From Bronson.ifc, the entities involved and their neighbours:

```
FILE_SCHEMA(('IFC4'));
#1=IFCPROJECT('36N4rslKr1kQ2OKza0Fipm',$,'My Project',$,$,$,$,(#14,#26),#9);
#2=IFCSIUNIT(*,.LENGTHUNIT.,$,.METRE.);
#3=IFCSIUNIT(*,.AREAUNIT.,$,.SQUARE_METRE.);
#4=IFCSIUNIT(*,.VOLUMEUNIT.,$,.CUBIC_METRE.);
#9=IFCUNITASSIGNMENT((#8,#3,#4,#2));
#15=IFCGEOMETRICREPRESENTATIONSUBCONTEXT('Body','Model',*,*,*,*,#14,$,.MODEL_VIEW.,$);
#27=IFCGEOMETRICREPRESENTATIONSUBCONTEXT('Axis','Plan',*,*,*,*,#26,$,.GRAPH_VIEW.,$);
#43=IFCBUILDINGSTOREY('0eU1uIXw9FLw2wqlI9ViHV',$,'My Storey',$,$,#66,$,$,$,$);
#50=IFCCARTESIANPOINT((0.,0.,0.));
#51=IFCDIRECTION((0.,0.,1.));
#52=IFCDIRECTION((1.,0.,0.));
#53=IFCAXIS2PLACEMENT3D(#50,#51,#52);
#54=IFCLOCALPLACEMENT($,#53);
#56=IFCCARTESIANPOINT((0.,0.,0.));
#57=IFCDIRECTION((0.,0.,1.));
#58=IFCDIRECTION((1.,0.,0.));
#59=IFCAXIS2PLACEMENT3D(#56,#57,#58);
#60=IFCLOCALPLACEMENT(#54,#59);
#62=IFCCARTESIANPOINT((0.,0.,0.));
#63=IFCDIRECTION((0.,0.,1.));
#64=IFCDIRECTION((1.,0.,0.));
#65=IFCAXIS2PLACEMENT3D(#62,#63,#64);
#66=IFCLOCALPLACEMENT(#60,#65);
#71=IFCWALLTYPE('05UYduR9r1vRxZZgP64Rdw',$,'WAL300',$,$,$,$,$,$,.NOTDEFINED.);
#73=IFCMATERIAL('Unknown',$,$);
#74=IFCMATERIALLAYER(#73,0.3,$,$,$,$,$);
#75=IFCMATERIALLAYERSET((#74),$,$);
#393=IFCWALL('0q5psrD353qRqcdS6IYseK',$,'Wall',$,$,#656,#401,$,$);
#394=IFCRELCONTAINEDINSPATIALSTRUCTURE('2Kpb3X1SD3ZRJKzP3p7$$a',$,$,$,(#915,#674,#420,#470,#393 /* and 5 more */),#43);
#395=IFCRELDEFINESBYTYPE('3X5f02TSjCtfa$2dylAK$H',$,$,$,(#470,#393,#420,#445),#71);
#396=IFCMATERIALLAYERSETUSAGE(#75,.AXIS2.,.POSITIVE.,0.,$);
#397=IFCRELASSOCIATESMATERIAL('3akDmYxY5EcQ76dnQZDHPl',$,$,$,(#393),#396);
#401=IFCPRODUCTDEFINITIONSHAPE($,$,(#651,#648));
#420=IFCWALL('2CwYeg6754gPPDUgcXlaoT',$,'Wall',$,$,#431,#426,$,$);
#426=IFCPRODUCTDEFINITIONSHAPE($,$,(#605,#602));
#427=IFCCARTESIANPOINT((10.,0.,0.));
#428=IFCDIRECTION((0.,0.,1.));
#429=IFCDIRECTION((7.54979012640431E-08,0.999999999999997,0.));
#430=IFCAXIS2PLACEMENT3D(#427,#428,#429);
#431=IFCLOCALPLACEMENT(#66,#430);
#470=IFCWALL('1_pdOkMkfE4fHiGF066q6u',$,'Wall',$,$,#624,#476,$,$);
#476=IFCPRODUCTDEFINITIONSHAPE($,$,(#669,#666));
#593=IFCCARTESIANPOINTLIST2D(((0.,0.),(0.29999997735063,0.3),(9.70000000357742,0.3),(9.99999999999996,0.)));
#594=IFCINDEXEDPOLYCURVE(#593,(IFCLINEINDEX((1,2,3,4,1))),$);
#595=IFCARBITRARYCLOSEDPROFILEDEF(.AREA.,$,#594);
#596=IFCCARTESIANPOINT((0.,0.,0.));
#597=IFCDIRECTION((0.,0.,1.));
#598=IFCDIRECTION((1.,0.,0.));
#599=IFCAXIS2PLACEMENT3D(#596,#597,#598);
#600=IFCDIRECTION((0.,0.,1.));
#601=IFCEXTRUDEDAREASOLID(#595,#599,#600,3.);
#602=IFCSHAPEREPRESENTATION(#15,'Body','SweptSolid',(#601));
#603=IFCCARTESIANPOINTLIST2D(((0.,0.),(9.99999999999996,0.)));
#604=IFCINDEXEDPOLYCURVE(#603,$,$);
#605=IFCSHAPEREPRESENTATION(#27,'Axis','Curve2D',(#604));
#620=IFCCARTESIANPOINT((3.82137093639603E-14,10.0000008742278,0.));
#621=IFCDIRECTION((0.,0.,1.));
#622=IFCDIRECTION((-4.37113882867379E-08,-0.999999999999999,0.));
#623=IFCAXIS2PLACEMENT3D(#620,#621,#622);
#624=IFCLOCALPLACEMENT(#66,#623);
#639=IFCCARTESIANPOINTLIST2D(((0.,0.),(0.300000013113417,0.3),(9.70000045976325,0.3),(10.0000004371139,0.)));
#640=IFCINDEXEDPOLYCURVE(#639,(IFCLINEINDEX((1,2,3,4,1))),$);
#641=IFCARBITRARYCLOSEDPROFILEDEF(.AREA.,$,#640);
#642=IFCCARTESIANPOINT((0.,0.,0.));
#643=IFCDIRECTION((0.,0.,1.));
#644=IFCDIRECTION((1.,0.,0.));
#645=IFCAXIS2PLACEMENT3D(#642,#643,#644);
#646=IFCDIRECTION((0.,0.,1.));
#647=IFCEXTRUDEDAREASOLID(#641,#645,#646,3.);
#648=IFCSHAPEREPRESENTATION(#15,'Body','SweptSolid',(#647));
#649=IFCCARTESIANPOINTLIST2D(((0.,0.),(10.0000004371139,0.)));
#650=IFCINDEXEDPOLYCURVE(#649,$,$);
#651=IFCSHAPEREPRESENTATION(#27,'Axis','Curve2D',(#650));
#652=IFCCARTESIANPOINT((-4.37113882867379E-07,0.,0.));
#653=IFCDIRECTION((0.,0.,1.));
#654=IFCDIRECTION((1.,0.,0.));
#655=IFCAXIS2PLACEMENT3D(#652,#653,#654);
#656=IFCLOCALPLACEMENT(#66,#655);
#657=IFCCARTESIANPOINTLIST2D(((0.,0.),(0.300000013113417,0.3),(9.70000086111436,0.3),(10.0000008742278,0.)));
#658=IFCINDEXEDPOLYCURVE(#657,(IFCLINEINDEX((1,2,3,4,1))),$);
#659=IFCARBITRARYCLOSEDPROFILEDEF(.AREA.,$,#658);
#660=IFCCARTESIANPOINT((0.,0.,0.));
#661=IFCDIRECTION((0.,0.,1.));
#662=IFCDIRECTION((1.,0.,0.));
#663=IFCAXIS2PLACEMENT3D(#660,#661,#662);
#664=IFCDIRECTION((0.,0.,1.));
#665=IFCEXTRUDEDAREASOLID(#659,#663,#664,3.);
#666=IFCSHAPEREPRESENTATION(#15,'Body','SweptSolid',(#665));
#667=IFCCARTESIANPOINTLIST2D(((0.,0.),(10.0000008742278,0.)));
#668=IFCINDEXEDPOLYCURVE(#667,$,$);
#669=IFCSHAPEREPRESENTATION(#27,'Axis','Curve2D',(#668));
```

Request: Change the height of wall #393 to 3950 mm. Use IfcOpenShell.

```python
import ifcopenshell
import ifcopenshell.geom
import ifcopenshell.util.representation
import ifcopenshell.util.shape
import ifcopenshell.util.unit

model = ifcopenshell.open("Bronson.ifc")
unit_scale = ifcopenshell.util.unit.calculate_unit_scale(model)
settings = ifcopenshell.geom.settings()


def volume(element):
    """Net volume in cubic metres, openings subtracted."""
    shape = ifcopenshell.geom.create_shape(settings, element)
    return ifcopenshell.util.shape.get_volume(shape.geometry)


wall = model.by_guid("0q5psrD353qRqcdS6IYseK")
before = volume(wall)

body = ifcopenshell.util.representation.get_representation(wall, "Model", "Body")
solid = body.Items[0]
old_height = solid.Depth
solid.Depth = 3.95 / unit_scale
after = volume(wall)

print(f"height {old_height:g} -> {solid.Depth:g}, volume {before:.3f} -> {after:.3f} m3")

model.write("Bronson_rev.ifc")
```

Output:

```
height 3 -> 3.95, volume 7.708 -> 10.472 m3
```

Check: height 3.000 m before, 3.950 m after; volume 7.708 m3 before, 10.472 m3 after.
